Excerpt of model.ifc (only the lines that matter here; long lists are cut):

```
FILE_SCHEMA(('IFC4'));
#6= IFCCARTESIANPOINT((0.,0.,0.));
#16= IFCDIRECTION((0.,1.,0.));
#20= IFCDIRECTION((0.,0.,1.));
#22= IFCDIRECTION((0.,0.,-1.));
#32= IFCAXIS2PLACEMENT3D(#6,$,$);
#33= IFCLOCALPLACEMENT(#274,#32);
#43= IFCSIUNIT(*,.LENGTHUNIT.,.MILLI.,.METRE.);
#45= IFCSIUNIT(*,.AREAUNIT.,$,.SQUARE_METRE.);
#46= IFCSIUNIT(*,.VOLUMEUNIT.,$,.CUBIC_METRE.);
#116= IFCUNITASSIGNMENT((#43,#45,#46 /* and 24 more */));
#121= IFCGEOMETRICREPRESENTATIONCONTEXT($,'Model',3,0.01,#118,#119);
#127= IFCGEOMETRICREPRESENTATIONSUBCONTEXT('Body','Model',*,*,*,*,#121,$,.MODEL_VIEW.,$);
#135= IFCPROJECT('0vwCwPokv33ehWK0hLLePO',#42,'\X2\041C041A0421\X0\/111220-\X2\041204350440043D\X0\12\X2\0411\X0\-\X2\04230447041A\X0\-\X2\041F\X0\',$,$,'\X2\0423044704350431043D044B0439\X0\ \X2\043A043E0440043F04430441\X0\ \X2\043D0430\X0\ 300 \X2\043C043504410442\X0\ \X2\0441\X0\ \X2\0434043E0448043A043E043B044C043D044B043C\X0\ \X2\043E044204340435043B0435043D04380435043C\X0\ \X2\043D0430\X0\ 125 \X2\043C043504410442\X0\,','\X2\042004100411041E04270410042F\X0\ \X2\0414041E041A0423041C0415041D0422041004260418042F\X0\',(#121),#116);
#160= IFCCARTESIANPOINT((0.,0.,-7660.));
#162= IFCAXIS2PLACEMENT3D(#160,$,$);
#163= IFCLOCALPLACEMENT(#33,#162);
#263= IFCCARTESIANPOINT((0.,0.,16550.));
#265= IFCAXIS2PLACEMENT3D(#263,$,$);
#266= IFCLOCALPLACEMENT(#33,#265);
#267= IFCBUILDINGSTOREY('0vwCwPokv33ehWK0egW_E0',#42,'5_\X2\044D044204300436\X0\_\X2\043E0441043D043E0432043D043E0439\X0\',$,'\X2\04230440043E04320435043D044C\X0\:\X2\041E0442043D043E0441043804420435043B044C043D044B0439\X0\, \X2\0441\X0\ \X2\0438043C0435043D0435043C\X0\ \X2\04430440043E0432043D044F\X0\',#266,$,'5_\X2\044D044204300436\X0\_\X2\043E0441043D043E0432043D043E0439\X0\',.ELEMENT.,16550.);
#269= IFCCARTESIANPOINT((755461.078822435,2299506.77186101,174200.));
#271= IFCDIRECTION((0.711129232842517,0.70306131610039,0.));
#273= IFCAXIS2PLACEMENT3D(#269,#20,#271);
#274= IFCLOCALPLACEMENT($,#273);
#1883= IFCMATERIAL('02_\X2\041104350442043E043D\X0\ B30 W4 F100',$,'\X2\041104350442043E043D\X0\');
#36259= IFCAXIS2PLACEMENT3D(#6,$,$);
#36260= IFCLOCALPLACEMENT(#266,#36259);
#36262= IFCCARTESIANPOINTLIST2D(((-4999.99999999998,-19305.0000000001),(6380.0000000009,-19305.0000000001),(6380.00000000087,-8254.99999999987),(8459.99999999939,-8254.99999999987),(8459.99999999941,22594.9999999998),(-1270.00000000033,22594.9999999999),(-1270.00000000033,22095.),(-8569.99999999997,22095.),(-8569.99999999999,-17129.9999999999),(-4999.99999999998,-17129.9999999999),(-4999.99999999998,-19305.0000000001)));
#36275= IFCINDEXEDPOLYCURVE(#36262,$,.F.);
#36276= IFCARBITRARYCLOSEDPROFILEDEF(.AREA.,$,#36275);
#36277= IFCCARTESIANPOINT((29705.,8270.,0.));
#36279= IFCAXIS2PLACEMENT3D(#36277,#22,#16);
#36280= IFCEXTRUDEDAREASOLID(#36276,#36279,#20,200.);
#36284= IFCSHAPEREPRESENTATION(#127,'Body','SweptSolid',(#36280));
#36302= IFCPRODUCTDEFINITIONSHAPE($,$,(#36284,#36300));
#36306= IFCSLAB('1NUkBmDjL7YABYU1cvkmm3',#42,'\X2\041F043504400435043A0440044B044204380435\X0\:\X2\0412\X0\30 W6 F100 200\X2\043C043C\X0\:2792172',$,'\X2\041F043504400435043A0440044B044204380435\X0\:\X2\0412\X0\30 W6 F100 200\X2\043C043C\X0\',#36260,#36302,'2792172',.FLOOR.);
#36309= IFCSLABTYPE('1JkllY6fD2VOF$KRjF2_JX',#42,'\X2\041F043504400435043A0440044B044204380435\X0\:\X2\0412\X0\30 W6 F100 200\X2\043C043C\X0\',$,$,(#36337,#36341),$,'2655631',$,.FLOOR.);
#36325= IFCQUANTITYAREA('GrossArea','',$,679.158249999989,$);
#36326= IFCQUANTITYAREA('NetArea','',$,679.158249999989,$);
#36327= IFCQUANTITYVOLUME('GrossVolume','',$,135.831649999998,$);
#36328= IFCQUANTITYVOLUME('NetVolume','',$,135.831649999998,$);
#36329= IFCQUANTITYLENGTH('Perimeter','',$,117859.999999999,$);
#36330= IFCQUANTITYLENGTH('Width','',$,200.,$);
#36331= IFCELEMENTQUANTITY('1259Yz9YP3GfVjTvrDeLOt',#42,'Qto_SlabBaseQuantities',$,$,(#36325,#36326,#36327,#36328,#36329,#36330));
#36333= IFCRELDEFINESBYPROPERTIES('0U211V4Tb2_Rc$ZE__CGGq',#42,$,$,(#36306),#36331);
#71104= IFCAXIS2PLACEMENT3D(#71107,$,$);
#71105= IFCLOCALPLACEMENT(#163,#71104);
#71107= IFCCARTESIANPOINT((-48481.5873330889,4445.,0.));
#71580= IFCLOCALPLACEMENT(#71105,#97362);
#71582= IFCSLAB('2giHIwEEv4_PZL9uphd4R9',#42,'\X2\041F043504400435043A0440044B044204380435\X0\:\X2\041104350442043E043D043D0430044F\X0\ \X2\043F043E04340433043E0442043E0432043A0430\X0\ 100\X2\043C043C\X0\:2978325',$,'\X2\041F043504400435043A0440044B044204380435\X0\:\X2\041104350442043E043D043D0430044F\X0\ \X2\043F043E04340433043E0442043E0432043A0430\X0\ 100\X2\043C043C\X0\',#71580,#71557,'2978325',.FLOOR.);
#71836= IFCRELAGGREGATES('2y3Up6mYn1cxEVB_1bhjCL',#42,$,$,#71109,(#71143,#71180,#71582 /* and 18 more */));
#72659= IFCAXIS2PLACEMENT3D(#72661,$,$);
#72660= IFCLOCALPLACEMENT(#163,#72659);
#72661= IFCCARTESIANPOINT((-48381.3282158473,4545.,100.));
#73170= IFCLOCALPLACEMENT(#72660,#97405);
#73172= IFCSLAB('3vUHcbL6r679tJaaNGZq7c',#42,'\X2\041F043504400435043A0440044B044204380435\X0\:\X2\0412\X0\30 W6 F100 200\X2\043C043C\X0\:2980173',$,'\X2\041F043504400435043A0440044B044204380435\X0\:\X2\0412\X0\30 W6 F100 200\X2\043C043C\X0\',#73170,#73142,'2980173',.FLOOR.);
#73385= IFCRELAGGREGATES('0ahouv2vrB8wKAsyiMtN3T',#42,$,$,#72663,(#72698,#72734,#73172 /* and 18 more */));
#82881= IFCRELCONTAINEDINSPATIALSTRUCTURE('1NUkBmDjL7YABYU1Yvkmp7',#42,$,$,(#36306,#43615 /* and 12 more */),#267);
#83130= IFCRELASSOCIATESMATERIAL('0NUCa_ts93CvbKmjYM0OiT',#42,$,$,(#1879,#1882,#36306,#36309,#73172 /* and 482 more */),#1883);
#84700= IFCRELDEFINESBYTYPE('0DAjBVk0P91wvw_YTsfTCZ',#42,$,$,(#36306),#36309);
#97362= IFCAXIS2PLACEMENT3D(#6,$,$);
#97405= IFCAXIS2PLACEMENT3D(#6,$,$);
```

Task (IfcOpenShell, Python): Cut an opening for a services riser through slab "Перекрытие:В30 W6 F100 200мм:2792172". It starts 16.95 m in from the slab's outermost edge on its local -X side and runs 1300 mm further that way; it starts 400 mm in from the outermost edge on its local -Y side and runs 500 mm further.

```python
import numpy as np
import ifcopenshell
import ifcopenshell.api.feature
import ifcopenshell.api.geometry
import ifcopenshell.api.pset
import ifcopenshell.api.root
import ifcopenshell.geom
import ifcopenshell.util.element
import ifcopenshell.util.placement
import ifcopenshell.util.representation
import ifcopenshell.util.shape
import ifcopenshell.util.unit

model = ifcopenshell.open("model.ifc")
unit_scale = ifcopenshell.util.unit.calculate_unit_scale(model)
area_scale = ifcopenshell.util.unit.calculate_unit_scale(model, "AREAUNIT")
volume_scale = ifcopenshell.util.unit.calculate_unit_scale(model, "VOLUMEUNIT")
settings = ifcopenshell.geom.settings()


def volume(element):
    """Net volume in cubic metres, openings subtracted."""
    shape = ifcopenshell.geom.create_shape(settings, element)
    return ifcopenshell.util.shape.get_volume(shape.geometry)


slab = model.by_guid("1NUkBmDjL7YABYU1cvkmm3")
before = volume(slab)

# Extent in the slab's own axes, in metres. The edges named are its -X and -Y sides.
slab_shape = ifcopenshell.geom.create_shape(settings, slab)
vertices = ifcopenshell.util.shape.get_vertices(slab_shape.geometry)
x_min, y_min, bottom = vertices.min(axis=0)
top = vertices[:, 2].max()

opening = ifcopenshell.api.root.create_entity(model, ifc_class="IfcOpeningElement", name="Services riser opening", predefined_type="OPENING")
context = ifcopenshell.util.representation.get_context(model, "Model", "Body", "MODEL_VIEW")
width, depth = 1.3, 0.5
outline = [(0.0, 0.0), (width, 0.0), (width, depth), (0.0, depth), (0.0, 0.0)]
# Overshoot both faces by 50 mm so the cut is clean.
shape = ifcopenshell.api.geometry.add_slab_representation(
    model, context=context, depth=top - bottom + 0.1, polyline=outline
)
ifcopenshell.api.geometry.assign_representation(model, product=opening, representation=shape)

matrix = ifcopenshell.util.placement.get_local_placement(slab.ObjectPlacement)
matrix[:, 3] = matrix @ np.append(np.array([x_min + 16.95, y_min + 0.4, bottom - 0.05]) / unit_scale, 1.0)
ifcopenshell.api.geometry.edit_object_placement(model, product=opening, matrix=matrix, is_si=False)
ifcopenshell.api.feature.add_feature(model, feature=opening, element=slab)

after = volume(slab)

# Update the slab's stored quantities.
qto = model.by_id(ifcopenshell.util.element.get_pset(slab, "Qto_SlabBaseQuantities", should_inherit=False)["id"])
ifcopenshell.api.pset.edit_qto(model, qto=qto, properties={
    "NetArea": after / (top - bottom) / area_scale,
    "NetVolume": after / volume_scale,
})

print(f"slab volume {before:.3f} -> {after:.3f} m3")

model.write("model-out.ifc")
```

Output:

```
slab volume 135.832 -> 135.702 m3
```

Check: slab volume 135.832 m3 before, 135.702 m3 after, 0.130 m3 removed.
